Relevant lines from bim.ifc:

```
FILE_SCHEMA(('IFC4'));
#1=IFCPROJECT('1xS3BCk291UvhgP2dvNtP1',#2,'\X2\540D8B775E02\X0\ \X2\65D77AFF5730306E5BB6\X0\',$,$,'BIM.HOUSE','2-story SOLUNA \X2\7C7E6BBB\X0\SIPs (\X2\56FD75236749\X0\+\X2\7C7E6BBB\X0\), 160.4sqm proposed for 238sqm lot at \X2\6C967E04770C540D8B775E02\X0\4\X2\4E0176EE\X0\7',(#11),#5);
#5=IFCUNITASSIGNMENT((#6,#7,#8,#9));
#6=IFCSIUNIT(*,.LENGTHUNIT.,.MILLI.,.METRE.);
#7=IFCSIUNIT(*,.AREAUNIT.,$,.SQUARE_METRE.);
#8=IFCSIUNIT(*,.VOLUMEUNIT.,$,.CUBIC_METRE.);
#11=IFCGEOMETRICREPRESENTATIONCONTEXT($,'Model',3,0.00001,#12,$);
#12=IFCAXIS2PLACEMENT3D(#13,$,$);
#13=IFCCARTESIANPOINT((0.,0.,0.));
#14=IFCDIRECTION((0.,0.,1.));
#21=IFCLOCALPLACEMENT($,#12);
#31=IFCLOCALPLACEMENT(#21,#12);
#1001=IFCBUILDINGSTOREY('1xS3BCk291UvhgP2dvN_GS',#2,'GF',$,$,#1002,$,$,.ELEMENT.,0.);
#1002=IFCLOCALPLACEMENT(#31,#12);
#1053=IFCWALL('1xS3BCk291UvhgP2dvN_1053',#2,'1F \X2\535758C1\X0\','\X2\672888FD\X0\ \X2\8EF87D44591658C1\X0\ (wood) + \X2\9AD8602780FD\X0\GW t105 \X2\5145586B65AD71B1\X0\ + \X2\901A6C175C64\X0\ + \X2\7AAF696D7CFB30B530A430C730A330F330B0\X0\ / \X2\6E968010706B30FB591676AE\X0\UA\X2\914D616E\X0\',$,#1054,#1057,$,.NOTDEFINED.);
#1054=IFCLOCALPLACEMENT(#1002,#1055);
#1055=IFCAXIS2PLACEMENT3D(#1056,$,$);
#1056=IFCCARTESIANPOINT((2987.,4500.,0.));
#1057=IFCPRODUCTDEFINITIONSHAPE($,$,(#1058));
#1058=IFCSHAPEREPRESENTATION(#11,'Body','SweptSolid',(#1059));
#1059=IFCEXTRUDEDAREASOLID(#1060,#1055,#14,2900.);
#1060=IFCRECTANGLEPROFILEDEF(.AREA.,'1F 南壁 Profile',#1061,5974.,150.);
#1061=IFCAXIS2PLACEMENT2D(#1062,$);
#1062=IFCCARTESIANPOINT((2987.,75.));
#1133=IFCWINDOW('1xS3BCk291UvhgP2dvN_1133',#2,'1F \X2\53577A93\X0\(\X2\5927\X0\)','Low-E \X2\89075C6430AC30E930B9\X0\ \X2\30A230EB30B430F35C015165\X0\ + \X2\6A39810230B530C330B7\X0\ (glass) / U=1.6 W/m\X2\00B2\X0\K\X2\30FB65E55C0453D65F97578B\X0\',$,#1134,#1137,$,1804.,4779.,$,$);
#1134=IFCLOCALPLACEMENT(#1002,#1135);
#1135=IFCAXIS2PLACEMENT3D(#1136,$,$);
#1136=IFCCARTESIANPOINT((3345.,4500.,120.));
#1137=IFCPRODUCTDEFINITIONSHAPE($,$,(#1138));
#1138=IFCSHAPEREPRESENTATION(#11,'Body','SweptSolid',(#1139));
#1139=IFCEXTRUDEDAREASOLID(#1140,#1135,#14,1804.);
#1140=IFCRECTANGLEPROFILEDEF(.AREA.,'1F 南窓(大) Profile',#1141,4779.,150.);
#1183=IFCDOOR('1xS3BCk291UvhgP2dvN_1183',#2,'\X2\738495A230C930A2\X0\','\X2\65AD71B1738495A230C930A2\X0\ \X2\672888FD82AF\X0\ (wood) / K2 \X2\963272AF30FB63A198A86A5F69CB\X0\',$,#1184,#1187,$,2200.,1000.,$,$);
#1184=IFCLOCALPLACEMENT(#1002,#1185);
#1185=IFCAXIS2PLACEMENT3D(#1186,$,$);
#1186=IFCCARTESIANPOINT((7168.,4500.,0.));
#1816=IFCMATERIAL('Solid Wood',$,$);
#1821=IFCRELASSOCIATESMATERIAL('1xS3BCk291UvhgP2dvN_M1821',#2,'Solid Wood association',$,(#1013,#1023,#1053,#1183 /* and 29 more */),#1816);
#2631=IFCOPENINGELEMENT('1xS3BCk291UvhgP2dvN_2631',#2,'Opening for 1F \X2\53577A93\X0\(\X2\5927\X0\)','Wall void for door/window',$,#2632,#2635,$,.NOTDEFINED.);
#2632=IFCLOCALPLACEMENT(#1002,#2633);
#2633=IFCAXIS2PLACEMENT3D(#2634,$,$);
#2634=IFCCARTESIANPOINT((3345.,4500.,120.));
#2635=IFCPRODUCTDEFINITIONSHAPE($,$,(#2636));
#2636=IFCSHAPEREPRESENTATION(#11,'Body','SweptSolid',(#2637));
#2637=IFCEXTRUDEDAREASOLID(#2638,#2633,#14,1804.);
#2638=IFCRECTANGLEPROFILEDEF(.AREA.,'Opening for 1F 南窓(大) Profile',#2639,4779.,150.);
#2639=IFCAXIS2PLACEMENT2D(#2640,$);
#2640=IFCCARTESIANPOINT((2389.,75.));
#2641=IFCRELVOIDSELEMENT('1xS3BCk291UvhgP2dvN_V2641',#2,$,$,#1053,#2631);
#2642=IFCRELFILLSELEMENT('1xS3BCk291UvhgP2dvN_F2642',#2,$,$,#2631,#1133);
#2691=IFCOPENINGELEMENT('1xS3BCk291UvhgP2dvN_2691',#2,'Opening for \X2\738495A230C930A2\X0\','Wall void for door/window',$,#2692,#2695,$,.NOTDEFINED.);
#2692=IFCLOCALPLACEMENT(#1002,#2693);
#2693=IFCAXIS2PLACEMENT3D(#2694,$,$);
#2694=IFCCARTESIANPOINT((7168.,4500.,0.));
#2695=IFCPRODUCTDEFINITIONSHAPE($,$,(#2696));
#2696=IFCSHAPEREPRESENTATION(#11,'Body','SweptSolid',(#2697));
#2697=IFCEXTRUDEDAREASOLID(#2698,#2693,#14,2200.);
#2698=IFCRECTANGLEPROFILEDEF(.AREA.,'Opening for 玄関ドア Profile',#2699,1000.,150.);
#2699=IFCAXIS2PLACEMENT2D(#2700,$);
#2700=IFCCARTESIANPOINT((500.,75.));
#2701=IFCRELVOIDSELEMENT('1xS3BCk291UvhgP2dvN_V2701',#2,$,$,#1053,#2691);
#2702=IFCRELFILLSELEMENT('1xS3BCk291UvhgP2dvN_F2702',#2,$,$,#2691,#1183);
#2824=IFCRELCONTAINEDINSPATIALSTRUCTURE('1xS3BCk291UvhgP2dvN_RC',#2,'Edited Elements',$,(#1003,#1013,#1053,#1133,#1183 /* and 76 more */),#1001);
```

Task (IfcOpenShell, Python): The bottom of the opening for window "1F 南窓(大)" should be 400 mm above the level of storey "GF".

```python
import numpy as np
import ifcopenshell
import ifcopenshell.api.geometry
import ifcopenshell.geom
import ifcopenshell.util.element
import ifcopenshell.util.placement
import ifcopenshell.util.shape
import ifcopenshell.util.unit

model = ifcopenshell.open("bim.ifc")
unit_scale = ifcopenshell.util.unit.calculate_unit_scale(model)

window = model.by_id(1133)
opening = window.FillsVoids[0].RelatingOpeningElement
storey = ifcopenshell.util.element.get_container(window, ifc_class="IfcBuildingStorey")
level = ifcopenshell.util.placement.get_local_placement(storey.ObjectPlacement)[2, 3]

# The opening's origin need not be at the sill, so measure its lowest point.
shape = ifcopenshell.geom.create_shape(ifcopenshell.geom.settings(), opening)
bottom = ifcopenshell.util.shape.get_shape_bottom_elevation(shape, shape.geometry) / unit_scale
dz = level + 400.0 - bottom

shift = np.array([0.0, 0.0, dz])
# The window is not placed relative to its opening, so move both.
for product in (opening, window):
    matrix = ifcopenshell.util.placement.get_local_placement(product.ObjectPlacement)
    matrix[:3, 3] += shift
    ifcopenshell.api.geometry.edit_object_placement(model, product=product, matrix=matrix, is_si=False)

print(f"moved by {dz * unit_scale:+.3f} m")

model.write("bim_v2.ifc")
```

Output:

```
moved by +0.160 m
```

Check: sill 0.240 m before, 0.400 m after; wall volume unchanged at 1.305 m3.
